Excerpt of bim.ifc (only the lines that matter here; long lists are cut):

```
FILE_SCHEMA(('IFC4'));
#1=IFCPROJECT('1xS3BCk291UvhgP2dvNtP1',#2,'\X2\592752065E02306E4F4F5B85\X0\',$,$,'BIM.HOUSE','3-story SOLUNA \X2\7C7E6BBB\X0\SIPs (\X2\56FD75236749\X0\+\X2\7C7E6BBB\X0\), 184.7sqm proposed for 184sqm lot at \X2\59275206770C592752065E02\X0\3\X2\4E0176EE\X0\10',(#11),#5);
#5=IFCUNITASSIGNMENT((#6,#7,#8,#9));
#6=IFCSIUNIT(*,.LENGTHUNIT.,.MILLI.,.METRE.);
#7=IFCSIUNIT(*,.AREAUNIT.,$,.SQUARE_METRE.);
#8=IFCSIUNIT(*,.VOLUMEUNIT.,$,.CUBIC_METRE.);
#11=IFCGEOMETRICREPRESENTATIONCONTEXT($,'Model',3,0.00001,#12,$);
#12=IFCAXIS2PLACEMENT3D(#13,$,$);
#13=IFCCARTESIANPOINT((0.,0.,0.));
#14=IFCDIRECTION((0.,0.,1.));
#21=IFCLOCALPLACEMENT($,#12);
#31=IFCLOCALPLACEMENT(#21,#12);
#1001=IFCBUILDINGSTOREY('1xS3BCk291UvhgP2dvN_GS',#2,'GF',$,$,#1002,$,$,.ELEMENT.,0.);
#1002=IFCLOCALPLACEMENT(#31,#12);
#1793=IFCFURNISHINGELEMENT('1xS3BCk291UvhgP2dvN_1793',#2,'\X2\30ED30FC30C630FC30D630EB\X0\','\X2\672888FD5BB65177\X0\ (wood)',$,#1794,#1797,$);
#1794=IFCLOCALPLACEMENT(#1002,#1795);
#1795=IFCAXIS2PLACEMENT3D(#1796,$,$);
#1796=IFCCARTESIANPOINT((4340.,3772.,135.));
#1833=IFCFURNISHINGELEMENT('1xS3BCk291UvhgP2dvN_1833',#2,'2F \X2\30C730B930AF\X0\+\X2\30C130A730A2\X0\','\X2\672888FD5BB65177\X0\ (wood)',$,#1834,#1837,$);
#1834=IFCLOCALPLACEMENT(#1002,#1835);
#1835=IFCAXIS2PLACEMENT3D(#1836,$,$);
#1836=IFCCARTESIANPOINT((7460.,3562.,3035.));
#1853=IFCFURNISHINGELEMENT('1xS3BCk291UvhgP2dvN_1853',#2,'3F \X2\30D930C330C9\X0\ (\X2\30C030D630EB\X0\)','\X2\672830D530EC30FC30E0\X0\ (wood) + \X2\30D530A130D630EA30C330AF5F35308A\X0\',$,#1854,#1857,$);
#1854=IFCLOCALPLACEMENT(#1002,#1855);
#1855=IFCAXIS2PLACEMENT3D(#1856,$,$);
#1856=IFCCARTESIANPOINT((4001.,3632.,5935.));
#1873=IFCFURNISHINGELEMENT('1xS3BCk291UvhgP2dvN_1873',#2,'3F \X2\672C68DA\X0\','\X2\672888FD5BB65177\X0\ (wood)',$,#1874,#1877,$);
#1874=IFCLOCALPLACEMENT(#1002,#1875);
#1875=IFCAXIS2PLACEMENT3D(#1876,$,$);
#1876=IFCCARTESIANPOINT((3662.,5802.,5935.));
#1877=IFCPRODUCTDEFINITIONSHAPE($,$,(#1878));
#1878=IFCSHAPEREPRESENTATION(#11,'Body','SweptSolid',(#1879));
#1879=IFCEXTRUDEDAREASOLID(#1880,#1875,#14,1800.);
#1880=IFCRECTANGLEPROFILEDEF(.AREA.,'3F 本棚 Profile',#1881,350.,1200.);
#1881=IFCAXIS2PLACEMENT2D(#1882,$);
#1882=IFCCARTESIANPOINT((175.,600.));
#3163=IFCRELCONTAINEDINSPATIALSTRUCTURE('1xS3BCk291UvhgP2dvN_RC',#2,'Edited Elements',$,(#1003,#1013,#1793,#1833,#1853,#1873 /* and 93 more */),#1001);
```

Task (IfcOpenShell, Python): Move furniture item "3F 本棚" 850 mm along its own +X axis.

```python
import ifcopenshell
import ifcopenshell.api.geometry
import ifcopenshell.util.placement
import ifcopenshell.util.unit

model = ifcopenshell.open("bim.ifc")
unit_scale = ifcopenshell.util.unit.calculate_unit_scale(model)

item = model.by_guid("1xS3BCk291UvhgP2dvN_1873")
matrix = ifcopenshell.util.placement.get_local_placement(item.ObjectPlacement)
matrix[:3, 3] += matrix[:3, 0] * 0.85 / unit_scale
ifcopenshell.api.geometry.edit_object_placement(model, product=item, matrix=matrix, is_si=False)

print(ifcopenshell.util.placement.get_local_placement(item.ObjectPlacement).round(3) + 0.0)

model.write("bim_v2.ifc")
```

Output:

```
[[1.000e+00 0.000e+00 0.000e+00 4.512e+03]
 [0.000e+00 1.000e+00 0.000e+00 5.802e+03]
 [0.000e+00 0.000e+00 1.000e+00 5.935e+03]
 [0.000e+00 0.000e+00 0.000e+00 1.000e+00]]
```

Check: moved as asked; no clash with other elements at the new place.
